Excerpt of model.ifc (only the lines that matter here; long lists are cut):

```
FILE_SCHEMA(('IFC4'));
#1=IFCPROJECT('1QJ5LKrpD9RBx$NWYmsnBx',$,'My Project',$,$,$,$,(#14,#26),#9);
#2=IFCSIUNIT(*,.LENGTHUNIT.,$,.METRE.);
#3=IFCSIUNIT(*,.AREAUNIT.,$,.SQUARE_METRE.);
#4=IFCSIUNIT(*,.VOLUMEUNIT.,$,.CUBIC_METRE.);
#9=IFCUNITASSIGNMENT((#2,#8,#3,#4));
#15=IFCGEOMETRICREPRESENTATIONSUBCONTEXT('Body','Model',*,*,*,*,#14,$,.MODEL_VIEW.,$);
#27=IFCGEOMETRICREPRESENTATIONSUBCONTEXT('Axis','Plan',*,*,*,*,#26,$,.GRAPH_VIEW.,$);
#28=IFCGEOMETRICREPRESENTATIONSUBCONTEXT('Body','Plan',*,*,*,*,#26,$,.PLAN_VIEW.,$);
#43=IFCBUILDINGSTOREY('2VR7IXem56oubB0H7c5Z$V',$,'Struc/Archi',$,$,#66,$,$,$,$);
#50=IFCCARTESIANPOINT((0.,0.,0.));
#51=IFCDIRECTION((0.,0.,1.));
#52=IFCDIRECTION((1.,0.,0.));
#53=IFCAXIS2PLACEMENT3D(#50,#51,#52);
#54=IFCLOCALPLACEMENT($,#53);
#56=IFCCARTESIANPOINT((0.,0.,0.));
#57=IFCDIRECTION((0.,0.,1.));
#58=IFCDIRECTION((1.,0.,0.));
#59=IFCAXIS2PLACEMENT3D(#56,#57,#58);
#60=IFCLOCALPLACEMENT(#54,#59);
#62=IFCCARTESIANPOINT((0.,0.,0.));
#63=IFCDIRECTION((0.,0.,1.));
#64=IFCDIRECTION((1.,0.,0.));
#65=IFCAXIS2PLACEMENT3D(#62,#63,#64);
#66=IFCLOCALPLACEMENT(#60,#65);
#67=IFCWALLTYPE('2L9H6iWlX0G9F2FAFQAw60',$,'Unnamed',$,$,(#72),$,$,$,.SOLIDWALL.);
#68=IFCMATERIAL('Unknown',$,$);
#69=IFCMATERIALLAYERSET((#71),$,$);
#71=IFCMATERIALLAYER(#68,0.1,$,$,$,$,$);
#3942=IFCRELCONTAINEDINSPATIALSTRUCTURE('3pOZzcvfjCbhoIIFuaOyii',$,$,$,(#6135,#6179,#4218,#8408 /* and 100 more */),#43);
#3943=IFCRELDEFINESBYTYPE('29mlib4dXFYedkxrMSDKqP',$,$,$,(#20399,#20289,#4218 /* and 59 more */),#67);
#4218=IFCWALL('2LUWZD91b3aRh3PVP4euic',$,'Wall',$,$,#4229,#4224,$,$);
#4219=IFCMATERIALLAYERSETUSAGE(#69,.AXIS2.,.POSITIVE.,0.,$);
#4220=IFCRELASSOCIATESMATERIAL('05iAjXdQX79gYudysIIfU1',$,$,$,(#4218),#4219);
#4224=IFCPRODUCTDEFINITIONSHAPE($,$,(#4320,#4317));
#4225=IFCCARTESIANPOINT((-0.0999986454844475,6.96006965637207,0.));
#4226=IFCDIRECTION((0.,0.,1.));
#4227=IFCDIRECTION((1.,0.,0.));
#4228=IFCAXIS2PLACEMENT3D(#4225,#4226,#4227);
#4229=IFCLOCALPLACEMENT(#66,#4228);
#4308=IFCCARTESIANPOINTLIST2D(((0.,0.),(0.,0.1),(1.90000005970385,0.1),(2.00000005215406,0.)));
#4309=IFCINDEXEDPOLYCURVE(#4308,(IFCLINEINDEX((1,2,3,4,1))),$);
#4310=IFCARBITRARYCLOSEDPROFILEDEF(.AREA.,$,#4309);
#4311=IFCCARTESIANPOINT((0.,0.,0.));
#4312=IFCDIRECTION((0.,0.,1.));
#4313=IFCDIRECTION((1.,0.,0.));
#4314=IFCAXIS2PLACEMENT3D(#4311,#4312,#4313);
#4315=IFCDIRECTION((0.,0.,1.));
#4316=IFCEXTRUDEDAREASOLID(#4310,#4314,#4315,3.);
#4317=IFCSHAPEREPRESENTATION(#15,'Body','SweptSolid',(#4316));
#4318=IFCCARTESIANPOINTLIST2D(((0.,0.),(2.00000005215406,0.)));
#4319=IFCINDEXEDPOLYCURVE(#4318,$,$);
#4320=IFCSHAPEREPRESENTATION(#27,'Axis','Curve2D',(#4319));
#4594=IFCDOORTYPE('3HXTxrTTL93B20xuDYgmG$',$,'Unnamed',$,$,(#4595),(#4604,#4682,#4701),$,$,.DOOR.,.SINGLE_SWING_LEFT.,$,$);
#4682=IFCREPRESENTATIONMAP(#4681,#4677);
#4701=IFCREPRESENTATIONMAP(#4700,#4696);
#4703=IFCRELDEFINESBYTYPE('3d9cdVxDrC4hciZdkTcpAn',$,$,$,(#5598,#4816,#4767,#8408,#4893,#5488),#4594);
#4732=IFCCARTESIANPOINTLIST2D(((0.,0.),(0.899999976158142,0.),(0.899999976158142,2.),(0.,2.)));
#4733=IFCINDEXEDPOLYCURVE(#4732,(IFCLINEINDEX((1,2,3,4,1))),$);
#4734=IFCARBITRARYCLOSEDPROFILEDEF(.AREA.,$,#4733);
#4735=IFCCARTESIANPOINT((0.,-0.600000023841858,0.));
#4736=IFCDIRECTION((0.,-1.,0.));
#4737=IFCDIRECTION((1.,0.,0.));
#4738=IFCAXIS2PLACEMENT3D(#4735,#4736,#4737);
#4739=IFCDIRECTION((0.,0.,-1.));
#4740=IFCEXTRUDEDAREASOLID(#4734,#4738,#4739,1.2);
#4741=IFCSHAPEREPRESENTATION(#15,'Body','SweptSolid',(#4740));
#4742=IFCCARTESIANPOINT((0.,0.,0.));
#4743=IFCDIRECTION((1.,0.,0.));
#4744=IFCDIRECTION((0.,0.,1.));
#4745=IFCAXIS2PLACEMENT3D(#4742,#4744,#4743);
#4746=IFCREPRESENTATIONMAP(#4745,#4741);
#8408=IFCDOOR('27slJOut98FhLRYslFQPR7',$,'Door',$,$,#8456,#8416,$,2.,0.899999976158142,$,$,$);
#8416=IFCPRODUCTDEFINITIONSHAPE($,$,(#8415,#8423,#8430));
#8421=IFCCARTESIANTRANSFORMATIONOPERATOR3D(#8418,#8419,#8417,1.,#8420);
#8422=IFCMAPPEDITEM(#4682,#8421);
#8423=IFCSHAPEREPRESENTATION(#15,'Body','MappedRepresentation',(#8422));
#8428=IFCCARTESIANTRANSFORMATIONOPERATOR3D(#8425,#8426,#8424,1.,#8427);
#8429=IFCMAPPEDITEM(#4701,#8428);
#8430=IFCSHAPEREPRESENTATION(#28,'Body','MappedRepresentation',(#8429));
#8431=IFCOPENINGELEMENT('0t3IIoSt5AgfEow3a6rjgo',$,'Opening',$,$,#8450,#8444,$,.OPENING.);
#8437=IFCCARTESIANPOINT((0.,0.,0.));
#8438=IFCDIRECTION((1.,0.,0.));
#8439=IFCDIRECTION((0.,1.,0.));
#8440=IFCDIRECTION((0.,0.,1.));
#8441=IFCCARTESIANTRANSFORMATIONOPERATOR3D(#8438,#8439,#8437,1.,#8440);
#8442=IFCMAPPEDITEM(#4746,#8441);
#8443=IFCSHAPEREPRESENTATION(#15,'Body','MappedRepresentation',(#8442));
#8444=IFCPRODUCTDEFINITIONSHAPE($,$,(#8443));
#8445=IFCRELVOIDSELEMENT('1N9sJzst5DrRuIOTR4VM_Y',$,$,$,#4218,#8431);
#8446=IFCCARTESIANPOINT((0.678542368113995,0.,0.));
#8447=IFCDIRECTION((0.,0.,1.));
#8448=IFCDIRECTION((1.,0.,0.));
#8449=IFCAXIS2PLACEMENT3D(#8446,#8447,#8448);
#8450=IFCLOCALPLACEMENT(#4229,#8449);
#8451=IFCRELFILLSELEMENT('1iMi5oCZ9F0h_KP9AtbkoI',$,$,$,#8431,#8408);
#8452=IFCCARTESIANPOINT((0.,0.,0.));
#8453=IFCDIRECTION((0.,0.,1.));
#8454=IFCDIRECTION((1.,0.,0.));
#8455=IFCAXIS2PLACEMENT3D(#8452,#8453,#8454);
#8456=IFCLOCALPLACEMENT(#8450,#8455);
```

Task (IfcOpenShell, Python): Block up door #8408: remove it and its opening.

```python
import ifcopenshell
import ifcopenshell.api.feature
import ifcopenshell.api.root
import ifcopenshell.geom
import ifcopenshell.util.shape

model = ifcopenshell.open("model.ifc")
settings = ifcopenshell.geom.settings()


def volume(element):
    """Net volume in cubic metres, openings subtracted."""
    shape = ifcopenshell.geom.create_shape(settings, element)
    return ifcopenshell.util.shape.get_volume(shape.geometry)


door = model.by_id(8408)
opening = door.FillsVoids[0].RelatingOpeningElement
wall = opening.VoidsElements[0].RelatingBuildingElement
before = volume(wall)

ifcopenshell.api.root.remove_product(model, product=door)
ifcopenshell.api.feature.remove_feature(model, feature=opening)

after = volume(wall)

print(f"wall volume {before:.3f} -> {after:.3f} m3")

model.write("model_updated.ifc")
```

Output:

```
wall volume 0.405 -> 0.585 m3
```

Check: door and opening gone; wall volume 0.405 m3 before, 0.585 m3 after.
